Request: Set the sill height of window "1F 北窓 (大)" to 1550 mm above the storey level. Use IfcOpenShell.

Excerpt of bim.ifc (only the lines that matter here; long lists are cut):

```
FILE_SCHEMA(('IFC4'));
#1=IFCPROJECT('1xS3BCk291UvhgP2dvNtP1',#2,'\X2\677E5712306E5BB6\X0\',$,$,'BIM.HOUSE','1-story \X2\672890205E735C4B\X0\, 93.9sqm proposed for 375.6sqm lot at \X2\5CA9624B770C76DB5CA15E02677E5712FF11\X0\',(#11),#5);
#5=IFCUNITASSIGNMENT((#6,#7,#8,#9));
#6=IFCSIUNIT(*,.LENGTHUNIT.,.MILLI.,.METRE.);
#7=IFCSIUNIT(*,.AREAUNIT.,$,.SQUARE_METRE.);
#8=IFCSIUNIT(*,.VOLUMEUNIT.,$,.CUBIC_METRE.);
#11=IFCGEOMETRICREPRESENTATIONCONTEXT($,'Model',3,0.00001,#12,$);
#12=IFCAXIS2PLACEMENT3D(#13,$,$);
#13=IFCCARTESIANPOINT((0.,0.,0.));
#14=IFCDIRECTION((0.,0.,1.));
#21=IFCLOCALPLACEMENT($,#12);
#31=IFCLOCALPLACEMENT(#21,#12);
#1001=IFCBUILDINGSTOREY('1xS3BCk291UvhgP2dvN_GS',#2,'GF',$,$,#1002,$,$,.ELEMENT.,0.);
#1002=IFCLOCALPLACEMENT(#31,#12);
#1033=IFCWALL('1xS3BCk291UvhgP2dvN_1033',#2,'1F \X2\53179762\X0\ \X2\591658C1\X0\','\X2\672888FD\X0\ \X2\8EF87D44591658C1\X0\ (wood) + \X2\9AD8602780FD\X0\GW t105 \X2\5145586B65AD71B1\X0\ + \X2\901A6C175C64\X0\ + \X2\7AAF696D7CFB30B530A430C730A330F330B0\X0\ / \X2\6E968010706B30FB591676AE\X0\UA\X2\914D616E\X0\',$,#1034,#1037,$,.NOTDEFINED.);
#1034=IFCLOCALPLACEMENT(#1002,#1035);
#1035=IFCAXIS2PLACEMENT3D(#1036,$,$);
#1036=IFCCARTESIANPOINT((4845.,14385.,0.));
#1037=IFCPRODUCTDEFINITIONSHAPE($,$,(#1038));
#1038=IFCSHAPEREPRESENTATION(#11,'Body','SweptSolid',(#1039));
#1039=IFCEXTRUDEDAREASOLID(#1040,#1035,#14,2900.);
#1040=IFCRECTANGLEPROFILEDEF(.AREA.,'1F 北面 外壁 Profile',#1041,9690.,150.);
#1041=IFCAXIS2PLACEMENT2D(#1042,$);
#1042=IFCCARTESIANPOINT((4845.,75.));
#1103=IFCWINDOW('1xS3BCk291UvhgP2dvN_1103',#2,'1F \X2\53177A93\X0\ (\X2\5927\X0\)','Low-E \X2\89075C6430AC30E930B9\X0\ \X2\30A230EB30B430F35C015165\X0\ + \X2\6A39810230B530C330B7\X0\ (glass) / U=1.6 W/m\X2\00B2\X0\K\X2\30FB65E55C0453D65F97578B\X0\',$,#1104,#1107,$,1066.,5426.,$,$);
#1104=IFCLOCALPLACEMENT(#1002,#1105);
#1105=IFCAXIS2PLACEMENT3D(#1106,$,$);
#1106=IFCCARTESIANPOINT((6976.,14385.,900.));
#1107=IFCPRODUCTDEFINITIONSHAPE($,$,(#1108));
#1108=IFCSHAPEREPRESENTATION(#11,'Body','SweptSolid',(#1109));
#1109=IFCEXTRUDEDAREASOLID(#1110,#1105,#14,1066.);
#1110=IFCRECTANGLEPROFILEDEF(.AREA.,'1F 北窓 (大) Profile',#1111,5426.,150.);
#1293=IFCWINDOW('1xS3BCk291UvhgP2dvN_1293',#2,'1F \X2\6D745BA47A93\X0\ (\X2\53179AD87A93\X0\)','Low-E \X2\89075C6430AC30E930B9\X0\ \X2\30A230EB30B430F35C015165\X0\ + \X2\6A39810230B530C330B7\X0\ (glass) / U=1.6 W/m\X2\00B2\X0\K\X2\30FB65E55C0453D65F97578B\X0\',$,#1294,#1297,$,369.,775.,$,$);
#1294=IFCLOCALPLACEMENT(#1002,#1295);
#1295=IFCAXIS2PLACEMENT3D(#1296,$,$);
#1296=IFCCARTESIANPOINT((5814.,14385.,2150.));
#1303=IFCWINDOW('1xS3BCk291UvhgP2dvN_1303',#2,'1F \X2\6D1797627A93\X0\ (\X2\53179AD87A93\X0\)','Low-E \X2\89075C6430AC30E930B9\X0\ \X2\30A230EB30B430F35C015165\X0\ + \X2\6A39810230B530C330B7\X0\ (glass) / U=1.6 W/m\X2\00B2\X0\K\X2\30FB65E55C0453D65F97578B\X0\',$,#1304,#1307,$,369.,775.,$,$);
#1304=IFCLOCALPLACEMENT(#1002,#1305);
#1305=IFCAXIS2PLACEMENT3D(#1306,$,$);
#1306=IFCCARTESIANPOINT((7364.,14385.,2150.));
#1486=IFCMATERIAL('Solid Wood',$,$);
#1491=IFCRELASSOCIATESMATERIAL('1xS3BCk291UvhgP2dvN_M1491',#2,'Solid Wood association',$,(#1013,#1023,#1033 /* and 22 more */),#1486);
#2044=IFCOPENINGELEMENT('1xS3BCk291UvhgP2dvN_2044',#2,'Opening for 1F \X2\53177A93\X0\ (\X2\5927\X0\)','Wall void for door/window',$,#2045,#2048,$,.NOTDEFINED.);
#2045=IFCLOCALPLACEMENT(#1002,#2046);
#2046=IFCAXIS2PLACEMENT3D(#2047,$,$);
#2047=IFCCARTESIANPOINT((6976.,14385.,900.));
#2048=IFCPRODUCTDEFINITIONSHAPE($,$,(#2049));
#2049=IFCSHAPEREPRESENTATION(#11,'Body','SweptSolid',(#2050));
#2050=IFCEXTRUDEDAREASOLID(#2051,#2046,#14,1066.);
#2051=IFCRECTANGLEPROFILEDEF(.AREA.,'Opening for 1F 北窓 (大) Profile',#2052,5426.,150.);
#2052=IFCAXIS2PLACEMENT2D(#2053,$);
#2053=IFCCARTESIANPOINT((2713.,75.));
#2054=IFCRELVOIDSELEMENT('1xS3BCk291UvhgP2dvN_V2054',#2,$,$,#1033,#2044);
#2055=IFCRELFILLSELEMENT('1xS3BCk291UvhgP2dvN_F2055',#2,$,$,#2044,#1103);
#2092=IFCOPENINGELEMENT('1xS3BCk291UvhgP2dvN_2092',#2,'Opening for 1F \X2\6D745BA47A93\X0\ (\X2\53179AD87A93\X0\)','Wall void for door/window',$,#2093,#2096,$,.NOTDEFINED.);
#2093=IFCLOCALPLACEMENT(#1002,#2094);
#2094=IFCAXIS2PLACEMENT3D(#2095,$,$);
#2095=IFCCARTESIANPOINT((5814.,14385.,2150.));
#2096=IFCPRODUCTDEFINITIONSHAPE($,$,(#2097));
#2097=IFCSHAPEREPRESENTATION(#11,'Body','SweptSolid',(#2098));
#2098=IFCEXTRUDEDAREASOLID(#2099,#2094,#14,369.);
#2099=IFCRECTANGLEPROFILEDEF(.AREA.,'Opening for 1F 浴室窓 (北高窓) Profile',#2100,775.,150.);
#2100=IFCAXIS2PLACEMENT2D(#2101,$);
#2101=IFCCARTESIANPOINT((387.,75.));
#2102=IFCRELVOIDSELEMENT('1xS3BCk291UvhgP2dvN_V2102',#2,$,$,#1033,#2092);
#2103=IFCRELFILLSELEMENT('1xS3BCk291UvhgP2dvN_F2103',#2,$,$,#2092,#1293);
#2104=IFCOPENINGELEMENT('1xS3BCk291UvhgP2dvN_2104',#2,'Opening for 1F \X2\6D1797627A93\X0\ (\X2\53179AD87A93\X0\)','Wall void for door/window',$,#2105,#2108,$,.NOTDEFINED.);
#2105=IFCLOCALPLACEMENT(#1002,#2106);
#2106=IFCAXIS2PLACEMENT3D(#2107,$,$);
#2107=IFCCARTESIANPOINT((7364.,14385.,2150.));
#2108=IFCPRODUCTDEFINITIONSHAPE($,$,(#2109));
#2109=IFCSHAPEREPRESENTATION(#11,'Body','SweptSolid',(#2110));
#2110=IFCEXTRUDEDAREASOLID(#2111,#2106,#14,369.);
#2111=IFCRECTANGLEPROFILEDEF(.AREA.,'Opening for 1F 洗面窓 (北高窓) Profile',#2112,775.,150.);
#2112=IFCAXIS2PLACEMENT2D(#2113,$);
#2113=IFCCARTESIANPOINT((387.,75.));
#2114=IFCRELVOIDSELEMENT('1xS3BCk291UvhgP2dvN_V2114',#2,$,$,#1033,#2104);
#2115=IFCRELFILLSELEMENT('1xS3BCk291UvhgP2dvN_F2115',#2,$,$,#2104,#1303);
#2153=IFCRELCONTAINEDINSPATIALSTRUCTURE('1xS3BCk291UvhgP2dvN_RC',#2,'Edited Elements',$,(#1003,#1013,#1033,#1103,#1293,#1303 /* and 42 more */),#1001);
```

```python
import numpy as np
import ifcopenshell
import ifcopenshell.api.geometry
import ifcopenshell.geom
import ifcopenshell.util.element
import ifcopenshell.util.placement
import ifcopenshell.util.shape
import ifcopenshell.util.unit

model = ifcopenshell.open("bim.ifc")
unit_scale = ifcopenshell.util.unit.calculate_unit_scale(model)

window = model.by_guid("1xS3BCk291UvhgP2dvN_1103")
opening = window.FillsVoids[0].RelatingOpeningElement
storey = ifcopenshell.util.element.get_container(window, ifc_class="IfcBuildingStorey")
level = ifcopenshell.util.placement.get_local_placement(storey.ObjectPlacement)[2, 3]

# The opening's origin need not be at the sill, so measure its lowest point.
shape = ifcopenshell.geom.create_shape(ifcopenshell.geom.settings(), opening)
bottom = ifcopenshell.util.shape.get_shape_bottom_elevation(shape, shape.geometry) / unit_scale
dz = level + 1.55 / unit_scale - bottom

shift = np.array([0.0, 0.0, dz])
# The window is not placed relative to its opening, so move both.
for product in (opening, window):
    matrix = ifcopenshell.util.placement.get_local_placement(product.ObjectPlacement)
    matrix[:3, 3] += shift
    ifcopenshell.api.geometry.edit_object_placement(model, product=product, matrix=matrix, is_si=False)

print(f"moved by {dz * unit_scale:+.3f} m")

model.write("bim_rev.ifc")
```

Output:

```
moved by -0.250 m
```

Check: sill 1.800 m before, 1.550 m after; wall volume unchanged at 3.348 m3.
